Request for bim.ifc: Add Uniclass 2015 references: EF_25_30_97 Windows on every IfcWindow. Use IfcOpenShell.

First a look at what the model holds.

```python
import ifcopenshell

model = ifcopenshell.open("bim.ifc")
print(model.schema)
print("classifications:", [c.Name for c in model.by_type("IfcClassification")])
for ifc_class in ("IfcDoor", "IfcRoof", "IfcStair", "IfcWall", "IfcWindow"):
    print(ifc_class, len(model.by_type(ifc_class)))
```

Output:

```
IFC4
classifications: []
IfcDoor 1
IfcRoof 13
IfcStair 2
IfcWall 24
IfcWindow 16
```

```python
import ifcopenshell
import ifcopenshell.api.classification

model = ifcopenshell.open("bim.ifc")

system = ifcopenshell.api.classification.add_classification(model, classification="Uniclass 2015")

codes = {
    "IfcWindow": ("EF_25_30_97", "Windows"),
}
for ifc_class, (code, name) in codes.items():
    products = model.by_type(ifc_class)
    ifcopenshell.api.classification.add_reference(
        model, products=products, classification=system, identification=code, name=name
    )
    print(code, len(products))

model.write("bim-out.ifc")
```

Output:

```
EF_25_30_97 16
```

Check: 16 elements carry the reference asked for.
